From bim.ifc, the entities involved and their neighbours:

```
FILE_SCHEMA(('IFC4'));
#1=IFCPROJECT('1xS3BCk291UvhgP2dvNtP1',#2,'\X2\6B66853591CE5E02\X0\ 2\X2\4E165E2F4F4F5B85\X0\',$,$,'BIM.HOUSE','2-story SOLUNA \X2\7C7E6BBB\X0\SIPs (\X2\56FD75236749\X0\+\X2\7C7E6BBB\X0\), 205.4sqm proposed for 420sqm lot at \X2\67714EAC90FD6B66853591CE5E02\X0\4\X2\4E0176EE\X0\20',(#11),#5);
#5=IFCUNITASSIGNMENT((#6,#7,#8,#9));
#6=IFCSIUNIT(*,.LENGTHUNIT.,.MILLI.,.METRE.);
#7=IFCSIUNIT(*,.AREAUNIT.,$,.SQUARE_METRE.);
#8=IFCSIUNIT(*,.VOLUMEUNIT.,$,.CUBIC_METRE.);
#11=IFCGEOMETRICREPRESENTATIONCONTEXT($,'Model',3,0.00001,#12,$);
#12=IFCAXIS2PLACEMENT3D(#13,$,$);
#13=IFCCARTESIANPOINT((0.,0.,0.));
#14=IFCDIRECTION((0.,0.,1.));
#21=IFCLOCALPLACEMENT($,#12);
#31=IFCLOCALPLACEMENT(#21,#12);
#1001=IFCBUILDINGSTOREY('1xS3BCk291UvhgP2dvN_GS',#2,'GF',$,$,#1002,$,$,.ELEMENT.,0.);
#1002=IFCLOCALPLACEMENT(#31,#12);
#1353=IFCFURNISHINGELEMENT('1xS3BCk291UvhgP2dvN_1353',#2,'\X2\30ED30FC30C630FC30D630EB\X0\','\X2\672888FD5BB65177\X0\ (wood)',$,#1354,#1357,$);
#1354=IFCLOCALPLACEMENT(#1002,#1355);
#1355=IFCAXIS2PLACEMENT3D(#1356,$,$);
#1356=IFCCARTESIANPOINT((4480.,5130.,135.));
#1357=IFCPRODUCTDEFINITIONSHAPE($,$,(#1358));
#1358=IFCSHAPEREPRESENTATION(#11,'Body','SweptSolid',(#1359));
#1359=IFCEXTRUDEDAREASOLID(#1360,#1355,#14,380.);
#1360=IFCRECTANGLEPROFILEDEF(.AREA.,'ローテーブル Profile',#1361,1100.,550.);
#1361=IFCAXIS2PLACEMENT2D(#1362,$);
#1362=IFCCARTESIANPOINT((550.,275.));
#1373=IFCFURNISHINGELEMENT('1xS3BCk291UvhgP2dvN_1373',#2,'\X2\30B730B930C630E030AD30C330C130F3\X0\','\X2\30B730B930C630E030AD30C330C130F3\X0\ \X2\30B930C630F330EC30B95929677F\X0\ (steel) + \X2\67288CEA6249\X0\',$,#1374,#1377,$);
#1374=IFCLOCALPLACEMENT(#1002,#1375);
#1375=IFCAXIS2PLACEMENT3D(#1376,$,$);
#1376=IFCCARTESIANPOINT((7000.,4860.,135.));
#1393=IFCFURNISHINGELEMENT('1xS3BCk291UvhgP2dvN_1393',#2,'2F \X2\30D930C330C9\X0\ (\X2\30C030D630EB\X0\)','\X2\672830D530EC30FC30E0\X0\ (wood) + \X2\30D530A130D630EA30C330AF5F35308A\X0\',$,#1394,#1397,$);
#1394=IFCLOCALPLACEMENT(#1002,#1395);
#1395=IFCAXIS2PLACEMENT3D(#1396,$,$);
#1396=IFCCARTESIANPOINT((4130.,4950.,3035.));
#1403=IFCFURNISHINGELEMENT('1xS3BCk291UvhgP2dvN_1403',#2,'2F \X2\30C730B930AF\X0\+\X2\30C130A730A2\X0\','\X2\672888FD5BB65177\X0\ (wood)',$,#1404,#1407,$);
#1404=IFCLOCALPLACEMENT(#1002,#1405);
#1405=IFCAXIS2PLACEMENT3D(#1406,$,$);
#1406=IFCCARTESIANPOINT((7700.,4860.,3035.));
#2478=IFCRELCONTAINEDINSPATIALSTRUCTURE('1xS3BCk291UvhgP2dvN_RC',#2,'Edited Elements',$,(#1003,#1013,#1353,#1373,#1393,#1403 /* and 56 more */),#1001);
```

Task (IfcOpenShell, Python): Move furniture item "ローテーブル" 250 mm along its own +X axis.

```python
import ifcopenshell
import ifcopenshell.api.geometry
import ifcopenshell.util.placement

model = ifcopenshell.open("bim.ifc")

item = model.by_guid("1xS3BCk291UvhgP2dvN_1353")
matrix = ifcopenshell.util.placement.get_local_placement(item.ObjectPlacement)
matrix[:3, 3] += matrix[:3, 0] * 250.0
ifcopenshell.api.geometry.edit_object_placement(model, product=item, matrix=matrix, is_si=False)

print(ifcopenshell.util.placement.get_local_placement(item.ObjectPlacement).round(3) + 0.0)

model.write("bim_rev.ifc")
```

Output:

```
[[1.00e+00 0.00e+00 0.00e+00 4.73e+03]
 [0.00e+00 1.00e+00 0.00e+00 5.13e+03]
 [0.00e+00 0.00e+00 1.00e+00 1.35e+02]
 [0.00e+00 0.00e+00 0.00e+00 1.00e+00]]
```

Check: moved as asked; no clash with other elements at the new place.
